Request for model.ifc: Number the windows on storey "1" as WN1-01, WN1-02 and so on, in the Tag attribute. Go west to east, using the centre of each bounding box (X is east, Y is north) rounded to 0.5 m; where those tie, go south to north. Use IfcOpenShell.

First a look at what the model holds.

```python
import ifcopenshell
import ifcopenshell.util.element
import ifcopenshell.util.placement

model = ifcopenshell.open("model.ifc")
print(model.schema)
storey = next(s for s in model.by_type("IfcBuildingStorey") if s.Name == "1")
windows = [e for e in ifcopenshell.util.element.get_decomposition(storey) if e.is_a("IfcWindow")]
for e in sorted(windows, key=lambda e: e.id()):
    origin = ifcopenshell.util.placement.get_local_placement(e.ObjectPlacement)[:3, 3]
    print(e.id(), e.Tag, e.Name, origin.round(2) + 0.0, sep=" | ")
```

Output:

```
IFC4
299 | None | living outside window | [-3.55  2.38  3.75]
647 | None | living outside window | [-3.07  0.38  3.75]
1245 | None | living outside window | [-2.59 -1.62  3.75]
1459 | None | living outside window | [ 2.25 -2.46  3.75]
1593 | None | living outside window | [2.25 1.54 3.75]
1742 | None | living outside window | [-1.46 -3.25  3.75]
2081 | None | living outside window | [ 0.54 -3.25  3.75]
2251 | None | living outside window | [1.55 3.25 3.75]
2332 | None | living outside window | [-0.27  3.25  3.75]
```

```python
import ifcopenshell
import ifcopenshell.geom
import ifcopenshell.util.element
import ifcopenshell.util.shape

model = ifcopenshell.open("model.ifc")
settings = ifcopenshell.geom.settings()
settings.set("use-world-coords", True)


def centre(element):
    shape = ifcopenshell.geom.create_shape(settings, element)
    return ifcopenshell.util.shape.get_bbox_centroid(shape.geometry)


storey = next(s for s in model.by_type("IfcBuildingStorey") if s.Name == "1")
windows = [e for e in ifcopenshell.util.element.get_decomposition(storey) if e.is_a("IfcWindow")]

# Insertion points can sit at a corner or the storey origin, so sort by the geometry (in metres).
centres = {e: centre(e) for e in windows}
windows.sort(key=lambda e: (round(centres[e][0] / 0.5), centres[e][1]))

for i, e in enumerate(windows, start=1):
    number = f"WN1-{i:02d}"
    e.Tag = number
    print(e.id(), number)

model.write("model_edited.ifc")
```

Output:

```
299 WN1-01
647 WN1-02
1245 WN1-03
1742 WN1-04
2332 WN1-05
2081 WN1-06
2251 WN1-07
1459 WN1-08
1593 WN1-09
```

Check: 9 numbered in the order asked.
